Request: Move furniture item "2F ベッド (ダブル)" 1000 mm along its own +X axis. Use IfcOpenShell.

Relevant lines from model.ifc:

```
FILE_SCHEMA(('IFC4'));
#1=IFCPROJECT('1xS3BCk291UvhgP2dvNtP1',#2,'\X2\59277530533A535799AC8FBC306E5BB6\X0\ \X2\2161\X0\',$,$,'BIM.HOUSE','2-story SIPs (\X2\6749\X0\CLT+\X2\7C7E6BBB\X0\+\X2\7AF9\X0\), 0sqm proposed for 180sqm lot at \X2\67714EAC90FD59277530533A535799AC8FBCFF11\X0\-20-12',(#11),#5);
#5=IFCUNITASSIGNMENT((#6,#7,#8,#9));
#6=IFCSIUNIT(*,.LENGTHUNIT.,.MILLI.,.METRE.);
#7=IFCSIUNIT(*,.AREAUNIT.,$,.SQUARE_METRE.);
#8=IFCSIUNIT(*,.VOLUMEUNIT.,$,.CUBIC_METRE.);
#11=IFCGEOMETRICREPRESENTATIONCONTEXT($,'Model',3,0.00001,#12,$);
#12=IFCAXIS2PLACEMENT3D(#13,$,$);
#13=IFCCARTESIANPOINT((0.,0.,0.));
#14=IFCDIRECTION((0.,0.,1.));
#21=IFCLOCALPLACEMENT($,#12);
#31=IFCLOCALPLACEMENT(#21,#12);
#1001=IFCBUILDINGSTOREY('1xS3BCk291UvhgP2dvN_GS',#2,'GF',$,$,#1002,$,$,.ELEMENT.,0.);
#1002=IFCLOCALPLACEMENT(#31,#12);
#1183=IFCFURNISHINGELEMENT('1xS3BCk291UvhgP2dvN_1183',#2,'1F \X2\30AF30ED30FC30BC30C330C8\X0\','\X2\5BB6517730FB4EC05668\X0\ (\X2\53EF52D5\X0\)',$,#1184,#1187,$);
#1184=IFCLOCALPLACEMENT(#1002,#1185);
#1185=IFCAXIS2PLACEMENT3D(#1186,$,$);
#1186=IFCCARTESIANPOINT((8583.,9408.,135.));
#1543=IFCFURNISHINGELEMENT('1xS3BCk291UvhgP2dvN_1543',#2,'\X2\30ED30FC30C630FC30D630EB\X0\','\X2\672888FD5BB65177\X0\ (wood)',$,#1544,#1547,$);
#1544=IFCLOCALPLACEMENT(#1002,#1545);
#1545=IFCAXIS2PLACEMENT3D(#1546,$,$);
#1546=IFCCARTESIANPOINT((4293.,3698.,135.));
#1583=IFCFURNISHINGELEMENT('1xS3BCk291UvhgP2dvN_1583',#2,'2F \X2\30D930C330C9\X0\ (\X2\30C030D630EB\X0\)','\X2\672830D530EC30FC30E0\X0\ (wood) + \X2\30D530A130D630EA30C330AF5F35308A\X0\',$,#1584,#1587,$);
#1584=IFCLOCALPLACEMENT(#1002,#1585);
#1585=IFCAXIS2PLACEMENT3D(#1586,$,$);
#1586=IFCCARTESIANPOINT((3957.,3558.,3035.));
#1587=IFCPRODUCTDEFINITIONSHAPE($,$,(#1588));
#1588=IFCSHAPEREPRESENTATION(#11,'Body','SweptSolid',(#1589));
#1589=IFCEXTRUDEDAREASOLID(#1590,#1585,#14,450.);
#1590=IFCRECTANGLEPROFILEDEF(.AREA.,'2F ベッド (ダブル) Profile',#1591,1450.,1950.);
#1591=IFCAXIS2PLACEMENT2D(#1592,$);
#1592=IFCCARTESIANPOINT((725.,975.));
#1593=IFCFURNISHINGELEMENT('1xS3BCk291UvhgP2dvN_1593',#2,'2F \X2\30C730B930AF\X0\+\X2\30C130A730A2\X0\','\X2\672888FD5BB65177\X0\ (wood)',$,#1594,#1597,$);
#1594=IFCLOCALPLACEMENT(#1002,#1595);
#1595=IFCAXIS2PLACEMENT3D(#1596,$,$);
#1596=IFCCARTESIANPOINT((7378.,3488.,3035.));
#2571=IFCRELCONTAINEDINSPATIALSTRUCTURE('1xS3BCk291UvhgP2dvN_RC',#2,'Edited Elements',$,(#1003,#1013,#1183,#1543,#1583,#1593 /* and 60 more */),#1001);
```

```python
import ifcopenshell
import ifcopenshell.api.geometry
import ifcopenshell.util.placement

model = ifcopenshell.open("model.ifc")

item = model.by_guid("1xS3BCk291UvhgP2dvN_1583")
matrix = ifcopenshell.util.placement.get_local_placement(item.ObjectPlacement)
matrix[:3, 3] += matrix[:3, 0] * 1000.0
ifcopenshell.api.geometry.edit_object_placement(model, product=item, matrix=matrix, is_si=False)

print(ifcopenshell.util.placement.get_local_placement(item.ObjectPlacement).round(3) + 0.0)

model.write("model_v2.ifc")
```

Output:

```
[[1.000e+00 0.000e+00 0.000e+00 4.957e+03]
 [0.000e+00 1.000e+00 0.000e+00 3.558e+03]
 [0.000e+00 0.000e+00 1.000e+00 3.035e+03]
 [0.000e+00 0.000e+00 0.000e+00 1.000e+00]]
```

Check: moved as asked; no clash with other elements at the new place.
